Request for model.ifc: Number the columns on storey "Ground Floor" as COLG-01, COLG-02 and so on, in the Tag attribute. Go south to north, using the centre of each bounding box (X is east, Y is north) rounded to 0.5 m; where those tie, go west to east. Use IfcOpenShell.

First a look at what the model holds.

```python
import ifcopenshell
import ifcopenshell.util.element
import ifcopenshell.util.placement

model = ifcopenshell.open("model.ifc")
print(model.schema)
storey = next(s for s in model.by_type("IfcBuildingStorey") if s.Name == "Ground Floor")
columns = [e for e in ifcopenshell.util.element.get_decomposition(storey) if e.is_a("IfcColumn")]
for e in sorted(columns, key=lambda e: e.id()):
    origin = ifcopenshell.util.placement.get_local_placement(e.ObjectPlacement)[:3, 3]
    print(e.id(), e.Tag, e.Name, origin.round(2) + 0.0, sep=" | ")
```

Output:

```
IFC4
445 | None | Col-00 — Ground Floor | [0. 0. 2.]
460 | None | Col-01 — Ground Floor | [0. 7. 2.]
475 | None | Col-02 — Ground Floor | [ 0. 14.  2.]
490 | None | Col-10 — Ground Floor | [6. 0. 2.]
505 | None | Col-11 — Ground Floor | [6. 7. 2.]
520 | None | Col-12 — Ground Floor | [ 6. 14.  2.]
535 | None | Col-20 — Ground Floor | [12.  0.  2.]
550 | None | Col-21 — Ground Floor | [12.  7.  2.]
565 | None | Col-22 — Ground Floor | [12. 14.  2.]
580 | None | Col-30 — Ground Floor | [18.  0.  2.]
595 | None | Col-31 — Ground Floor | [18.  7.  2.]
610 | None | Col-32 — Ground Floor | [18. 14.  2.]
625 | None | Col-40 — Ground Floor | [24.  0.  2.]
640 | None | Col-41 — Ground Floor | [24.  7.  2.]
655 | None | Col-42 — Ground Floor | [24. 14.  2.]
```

```python
import ifcopenshell
import ifcopenshell.geom
import ifcopenshell.util.element
import ifcopenshell.util.shape

model = ifcopenshell.open("model.ifc")
settings = ifcopenshell.geom.settings()
settings.set("use-world-coords", True)


def centre(element):
    shape = ifcopenshell.geom.create_shape(settings, element)
    return ifcopenshell.util.shape.get_bbox_centroid(shape.geometry)


storey = next(s for s in model.by_type("IfcBuildingStorey") if s.Name == "Ground Floor")
columns = [e for e in ifcopenshell.util.element.get_decomposition(storey) if e.is_a("IfcColumn")]

# Insertion points can sit at a corner or the storey origin, so sort by the geometry (in metres).
centres = {e: centre(e) for e in columns}
columns.sort(key=lambda e: (round(centres[e][1] / 0.5), centres[e][0]))

for i, e in enumerate(columns, start=1):
    number = f"COLG-{i:02d}"
    e.Tag = number
    print(e.id(), number)

model.write("model_rev.ifc")
```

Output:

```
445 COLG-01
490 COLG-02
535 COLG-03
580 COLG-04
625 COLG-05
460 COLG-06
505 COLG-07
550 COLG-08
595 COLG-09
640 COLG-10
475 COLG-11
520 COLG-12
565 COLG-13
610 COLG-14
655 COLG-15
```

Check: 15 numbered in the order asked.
